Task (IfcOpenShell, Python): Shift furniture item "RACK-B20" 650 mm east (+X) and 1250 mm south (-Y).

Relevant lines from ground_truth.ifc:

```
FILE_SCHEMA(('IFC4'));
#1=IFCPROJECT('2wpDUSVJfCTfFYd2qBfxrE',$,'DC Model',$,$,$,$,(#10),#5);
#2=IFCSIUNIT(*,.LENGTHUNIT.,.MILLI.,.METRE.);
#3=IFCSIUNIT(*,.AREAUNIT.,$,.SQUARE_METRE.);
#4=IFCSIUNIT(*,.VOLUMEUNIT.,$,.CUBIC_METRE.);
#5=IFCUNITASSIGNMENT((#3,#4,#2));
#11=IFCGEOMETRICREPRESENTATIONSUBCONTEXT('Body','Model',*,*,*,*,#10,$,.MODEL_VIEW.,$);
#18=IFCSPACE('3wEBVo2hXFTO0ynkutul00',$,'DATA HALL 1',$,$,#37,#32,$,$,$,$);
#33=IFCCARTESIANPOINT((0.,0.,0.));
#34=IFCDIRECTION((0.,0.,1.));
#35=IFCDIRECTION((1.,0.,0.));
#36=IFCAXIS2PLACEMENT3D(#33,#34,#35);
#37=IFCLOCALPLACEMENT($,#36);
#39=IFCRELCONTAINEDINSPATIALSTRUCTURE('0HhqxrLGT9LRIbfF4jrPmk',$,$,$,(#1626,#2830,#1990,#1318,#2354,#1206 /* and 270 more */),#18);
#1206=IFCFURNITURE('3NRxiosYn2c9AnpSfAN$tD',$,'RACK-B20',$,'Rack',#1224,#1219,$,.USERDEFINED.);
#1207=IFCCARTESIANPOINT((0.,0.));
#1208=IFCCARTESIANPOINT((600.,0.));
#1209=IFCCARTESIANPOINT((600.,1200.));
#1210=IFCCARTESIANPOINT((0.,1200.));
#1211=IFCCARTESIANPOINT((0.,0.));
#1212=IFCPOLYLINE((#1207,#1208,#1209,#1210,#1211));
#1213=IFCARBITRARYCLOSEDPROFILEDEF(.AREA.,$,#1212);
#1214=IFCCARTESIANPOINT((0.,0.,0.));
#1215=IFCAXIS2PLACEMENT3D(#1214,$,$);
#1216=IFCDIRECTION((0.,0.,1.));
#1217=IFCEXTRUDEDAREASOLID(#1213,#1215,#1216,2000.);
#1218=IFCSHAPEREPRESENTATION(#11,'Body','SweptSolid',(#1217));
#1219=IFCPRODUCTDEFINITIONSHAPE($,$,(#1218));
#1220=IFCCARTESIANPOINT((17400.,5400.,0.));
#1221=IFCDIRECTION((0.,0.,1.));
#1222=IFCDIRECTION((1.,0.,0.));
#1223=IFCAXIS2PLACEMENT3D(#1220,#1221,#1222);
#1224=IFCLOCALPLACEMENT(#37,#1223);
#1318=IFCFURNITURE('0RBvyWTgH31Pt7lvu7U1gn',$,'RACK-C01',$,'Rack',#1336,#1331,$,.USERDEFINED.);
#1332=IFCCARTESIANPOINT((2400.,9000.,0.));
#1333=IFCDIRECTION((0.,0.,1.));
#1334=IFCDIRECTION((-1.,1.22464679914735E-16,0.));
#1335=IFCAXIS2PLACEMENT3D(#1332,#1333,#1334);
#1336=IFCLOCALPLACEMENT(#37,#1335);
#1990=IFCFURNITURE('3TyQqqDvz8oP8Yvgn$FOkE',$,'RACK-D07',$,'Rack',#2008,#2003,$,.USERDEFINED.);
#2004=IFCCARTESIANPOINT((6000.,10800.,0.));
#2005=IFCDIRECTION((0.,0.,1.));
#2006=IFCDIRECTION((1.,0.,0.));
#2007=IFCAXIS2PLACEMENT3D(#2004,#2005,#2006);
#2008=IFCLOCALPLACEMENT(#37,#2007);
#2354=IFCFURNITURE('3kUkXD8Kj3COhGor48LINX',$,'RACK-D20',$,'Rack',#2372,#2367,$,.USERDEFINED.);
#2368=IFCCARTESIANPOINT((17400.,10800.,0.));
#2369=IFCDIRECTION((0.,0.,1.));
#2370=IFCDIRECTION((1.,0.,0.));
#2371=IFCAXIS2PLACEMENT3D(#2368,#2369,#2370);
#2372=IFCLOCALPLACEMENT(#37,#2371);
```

```python
import ifcopenshell
import ifcopenshell.api.geometry
import ifcopenshell.util.placement

model = ifcopenshell.open("ground_truth.ifc")

item = model.by_guid("3NRxiosYn2c9AnpSfAN$tD")
matrix = ifcopenshell.util.placement.get_local_placement(item.ObjectPlacement)
matrix[0, 3] += 650.0
matrix[1, 3] -= 1250.0
ifcopenshell.api.geometry.edit_object_placement(model, product=item, matrix=matrix, is_si=False)

print(ifcopenshell.util.placement.get_local_placement(item.ObjectPlacement).round(3) + 0.0)

model.write("ground_truth_updated.ifc")
```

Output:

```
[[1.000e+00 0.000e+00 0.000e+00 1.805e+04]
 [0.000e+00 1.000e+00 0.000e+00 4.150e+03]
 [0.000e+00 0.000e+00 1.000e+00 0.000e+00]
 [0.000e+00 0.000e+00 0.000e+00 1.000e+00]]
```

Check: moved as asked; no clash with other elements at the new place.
